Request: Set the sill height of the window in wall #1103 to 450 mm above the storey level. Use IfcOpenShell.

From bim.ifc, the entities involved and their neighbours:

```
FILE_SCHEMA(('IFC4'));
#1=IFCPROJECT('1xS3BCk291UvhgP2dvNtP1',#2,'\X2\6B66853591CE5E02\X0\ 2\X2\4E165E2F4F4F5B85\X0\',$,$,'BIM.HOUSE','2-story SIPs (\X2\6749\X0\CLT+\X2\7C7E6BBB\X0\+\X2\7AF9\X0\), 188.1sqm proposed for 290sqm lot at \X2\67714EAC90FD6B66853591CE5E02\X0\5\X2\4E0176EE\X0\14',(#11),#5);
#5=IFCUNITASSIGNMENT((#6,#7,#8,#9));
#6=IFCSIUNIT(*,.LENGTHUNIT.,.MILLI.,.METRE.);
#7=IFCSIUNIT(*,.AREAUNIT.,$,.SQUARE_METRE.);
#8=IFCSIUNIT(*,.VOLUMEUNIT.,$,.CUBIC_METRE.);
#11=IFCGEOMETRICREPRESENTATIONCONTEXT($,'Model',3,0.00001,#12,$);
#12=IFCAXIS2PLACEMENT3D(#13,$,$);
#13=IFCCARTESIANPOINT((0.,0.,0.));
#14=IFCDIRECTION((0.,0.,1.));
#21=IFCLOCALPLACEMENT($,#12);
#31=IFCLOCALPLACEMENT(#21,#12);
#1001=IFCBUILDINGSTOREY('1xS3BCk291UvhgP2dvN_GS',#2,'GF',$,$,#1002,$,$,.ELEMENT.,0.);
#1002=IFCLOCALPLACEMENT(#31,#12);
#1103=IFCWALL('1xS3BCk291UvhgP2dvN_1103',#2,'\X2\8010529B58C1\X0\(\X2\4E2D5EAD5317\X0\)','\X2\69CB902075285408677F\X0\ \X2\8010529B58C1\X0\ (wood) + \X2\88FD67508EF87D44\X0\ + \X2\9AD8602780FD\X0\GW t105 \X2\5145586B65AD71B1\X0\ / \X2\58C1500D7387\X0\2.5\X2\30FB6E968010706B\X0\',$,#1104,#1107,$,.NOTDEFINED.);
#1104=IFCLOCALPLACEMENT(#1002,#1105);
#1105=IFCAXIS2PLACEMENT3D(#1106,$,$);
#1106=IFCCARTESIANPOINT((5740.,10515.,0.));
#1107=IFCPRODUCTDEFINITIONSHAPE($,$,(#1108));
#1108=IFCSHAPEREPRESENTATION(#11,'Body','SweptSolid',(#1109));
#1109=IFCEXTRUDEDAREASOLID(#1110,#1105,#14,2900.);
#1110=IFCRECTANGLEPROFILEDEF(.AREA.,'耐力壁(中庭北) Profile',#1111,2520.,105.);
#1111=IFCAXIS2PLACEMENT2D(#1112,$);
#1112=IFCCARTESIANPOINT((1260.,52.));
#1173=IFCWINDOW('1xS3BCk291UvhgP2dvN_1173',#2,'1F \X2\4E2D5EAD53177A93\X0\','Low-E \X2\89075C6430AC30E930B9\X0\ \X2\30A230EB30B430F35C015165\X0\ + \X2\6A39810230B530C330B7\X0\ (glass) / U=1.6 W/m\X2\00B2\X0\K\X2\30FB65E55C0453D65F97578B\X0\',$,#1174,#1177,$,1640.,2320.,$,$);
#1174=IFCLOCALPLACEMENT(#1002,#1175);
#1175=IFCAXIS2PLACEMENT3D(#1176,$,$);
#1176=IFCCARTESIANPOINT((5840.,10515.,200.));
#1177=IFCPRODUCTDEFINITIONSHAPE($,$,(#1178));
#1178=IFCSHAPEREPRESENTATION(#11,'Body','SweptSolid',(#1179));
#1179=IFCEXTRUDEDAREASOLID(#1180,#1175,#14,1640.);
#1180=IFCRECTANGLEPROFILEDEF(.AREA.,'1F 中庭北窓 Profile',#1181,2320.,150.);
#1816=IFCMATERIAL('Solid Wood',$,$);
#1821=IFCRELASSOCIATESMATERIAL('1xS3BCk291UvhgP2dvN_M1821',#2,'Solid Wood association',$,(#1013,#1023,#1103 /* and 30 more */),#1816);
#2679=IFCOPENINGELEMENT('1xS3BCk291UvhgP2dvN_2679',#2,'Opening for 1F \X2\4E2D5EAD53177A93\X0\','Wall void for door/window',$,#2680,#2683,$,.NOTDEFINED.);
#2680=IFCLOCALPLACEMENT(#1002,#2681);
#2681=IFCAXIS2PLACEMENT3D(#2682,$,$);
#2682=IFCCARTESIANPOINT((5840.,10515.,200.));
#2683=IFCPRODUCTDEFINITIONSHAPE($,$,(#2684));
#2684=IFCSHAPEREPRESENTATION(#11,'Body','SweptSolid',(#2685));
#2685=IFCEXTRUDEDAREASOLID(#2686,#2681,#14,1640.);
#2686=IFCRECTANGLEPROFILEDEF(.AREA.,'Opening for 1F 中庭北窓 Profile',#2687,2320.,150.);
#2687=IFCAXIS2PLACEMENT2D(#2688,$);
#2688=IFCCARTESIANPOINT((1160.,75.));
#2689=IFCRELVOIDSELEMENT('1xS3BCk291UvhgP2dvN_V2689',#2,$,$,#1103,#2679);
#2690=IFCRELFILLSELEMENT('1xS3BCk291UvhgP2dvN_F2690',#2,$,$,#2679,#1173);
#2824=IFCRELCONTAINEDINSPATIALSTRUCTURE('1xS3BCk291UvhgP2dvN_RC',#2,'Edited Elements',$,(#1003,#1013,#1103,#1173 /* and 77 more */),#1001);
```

```python
import numpy as np
import ifcopenshell
import ifcopenshell.api.geometry
import ifcopenshell.geom
import ifcopenshell.util.element
import ifcopenshell.util.placement
import ifcopenshell.util.shape
import ifcopenshell.util.unit

model = ifcopenshell.open("bim.ifc")
unit_scale = ifcopenshell.util.unit.calculate_unit_scale(model)

window = model.by_id(1173)
opening = window.FillsVoids[0].RelatingOpeningElement
storey = ifcopenshell.util.element.get_container(window, ifc_class="IfcBuildingStorey")
level = ifcopenshell.util.placement.get_local_placement(storey.ObjectPlacement)[2, 3]

# The opening's origin need not be at the sill, so measure its lowest point.
shape = ifcopenshell.geom.create_shape(ifcopenshell.geom.settings(), opening)
bottom = ifcopenshell.util.shape.get_shape_bottom_elevation(shape, shape.geometry) / unit_scale
dz = level + 450.0 - bottom

shift = np.array([0.0, 0.0, dz])
# The window is not placed relative to its opening, so move both.
for product in (opening, window):
    matrix = ifcopenshell.util.placement.get_local_placement(product.ObjectPlacement)
    matrix[:3, 3] += shift
    ifcopenshell.api.geometry.edit_object_placement(model, product=product, matrix=matrix, is_si=False)

print(f"moved by {dz * unit_scale:+.3f} m")

model.write("bim-out.ifc")
```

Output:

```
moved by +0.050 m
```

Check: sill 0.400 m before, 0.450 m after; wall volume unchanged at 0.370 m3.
